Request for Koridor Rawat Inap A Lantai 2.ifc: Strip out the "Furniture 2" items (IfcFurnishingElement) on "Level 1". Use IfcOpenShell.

First a look at what the model holds.

```python
import ifcopenshell
import ifcopenshell.util.element

model = ifcopenshell.open("Koridor Rawat Inap A Lantai 2.ifc")
print(model.schema)
storey = next(s for s in model.by_type("IfcBuildingStorey") if s.Name == "Level 1")
furniture = [e for e in ifcopenshell.util.element.get_decomposition(storey) if e.is_a("IfcFurnishingElement")]
seen = {}
for e in furniture:
    element_type = ifcopenshell.util.element.get_type(e)
    name = element_type.Name if element_type not in (None, e) else None
    seen[name] = seen.get(name, 0) + 1
for name, count in sorted(seen.items(), key=str):
    print(count, "x", name)
```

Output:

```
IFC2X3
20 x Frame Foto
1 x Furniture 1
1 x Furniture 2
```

```python
import ifcopenshell
import ifcopenshell.api.root
import ifcopenshell.util.element

model = ifcopenshell.open("Koridor Rawat Inap A Lantai 2.ifc")

storey = next(s for s in model.by_type("IfcBuildingStorey") if s.Name == "Level 1")
furniture = [e for e in ifcopenshell.util.element.get_decomposition(storey) if e.is_a("IfcFurnishingElement")]
targets = [e for e in furniture if (t := ifcopenshell.util.element.get_type(e)) not in (None, e) and t.Name == "Furniture 2"]

for e in targets:
    ifcopenshell.api.root.remove_product(model, product=e)
print(len(targets), "removed")

model.write("Koridor Rawat Inap A Lantai 2_edited.ifc")
```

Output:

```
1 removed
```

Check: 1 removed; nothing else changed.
